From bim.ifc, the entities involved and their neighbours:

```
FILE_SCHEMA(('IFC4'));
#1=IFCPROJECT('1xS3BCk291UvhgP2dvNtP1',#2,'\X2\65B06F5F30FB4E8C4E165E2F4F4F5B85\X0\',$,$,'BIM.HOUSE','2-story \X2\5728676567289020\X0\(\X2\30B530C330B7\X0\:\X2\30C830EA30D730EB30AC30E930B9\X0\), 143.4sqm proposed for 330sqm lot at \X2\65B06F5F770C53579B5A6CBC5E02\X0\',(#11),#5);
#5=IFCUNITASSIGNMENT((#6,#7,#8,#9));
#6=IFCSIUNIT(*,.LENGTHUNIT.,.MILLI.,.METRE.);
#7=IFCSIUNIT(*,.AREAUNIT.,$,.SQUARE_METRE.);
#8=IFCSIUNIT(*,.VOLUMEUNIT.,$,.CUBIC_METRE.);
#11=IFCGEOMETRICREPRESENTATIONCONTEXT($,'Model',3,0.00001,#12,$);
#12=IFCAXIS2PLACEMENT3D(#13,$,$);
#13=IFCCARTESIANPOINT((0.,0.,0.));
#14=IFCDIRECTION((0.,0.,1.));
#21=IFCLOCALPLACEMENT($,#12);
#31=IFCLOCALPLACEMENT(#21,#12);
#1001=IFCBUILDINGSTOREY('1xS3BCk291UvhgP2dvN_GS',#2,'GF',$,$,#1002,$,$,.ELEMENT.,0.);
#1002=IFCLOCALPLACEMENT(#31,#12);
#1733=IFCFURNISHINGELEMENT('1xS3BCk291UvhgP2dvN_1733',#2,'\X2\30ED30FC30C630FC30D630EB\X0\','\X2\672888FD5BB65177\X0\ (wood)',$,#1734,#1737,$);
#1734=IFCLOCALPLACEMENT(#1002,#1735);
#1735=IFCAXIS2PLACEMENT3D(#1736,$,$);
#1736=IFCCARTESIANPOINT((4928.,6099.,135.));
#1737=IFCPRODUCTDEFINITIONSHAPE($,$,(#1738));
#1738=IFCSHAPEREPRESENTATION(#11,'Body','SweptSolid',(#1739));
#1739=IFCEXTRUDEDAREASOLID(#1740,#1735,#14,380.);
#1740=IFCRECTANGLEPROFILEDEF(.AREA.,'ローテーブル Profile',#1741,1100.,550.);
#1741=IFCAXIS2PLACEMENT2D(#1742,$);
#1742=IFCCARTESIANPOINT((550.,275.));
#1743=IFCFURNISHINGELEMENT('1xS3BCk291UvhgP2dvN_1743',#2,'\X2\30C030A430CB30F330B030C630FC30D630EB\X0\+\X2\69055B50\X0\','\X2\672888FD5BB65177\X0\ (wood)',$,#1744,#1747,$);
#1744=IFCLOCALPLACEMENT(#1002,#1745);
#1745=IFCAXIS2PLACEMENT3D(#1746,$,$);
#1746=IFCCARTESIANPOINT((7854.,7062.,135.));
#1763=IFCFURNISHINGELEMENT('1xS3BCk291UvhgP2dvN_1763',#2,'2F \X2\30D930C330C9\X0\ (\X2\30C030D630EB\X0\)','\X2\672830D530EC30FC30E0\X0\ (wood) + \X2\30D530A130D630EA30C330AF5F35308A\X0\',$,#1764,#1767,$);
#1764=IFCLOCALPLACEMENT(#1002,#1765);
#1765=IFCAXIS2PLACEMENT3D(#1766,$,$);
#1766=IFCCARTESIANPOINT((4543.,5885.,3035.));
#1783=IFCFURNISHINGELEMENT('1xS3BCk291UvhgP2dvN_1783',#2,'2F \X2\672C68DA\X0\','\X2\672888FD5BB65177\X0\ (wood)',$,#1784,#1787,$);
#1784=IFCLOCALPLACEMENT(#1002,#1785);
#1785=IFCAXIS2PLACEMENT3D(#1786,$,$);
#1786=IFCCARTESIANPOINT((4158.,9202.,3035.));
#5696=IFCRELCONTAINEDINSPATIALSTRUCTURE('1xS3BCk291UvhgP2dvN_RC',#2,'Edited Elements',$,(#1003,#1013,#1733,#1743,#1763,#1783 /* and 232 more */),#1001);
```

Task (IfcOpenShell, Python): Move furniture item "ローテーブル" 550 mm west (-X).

```python
import ifcopenshell
import ifcopenshell.api.geometry
import ifcopenshell.util.placement
import ifcopenshell.util.unit

model = ifcopenshell.open("bim.ifc")
unit_scale = ifcopenshell.util.unit.calculate_unit_scale(model)

item = model.by_guid("1xS3BCk291UvhgP2dvN_1733")
matrix = ifcopenshell.util.placement.get_local_placement(item.ObjectPlacement)
matrix[0, 3] -= 0.55 / unit_scale
ifcopenshell.api.geometry.edit_object_placement(model, product=item, matrix=matrix, is_si=False)

print(ifcopenshell.util.placement.get_local_placement(item.ObjectPlacement).round(3) + 0.0)

model.write("bim_updated.ifc")
```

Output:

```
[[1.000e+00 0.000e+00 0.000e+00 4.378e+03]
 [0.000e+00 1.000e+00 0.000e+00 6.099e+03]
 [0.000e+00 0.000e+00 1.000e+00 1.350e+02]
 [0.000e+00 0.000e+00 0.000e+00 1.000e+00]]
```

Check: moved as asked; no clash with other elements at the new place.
